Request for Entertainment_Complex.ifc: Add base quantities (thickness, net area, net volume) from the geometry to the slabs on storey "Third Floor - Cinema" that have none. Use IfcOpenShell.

First a look at what the model holds.

```python
import ifcopenshell
import ifcopenshell.util.element
import ifcopenshell.util.unit

model = ifcopenshell.open("Entertainment_Complex.ifc")
print(model.schema)
for unit_type in ("LENGTHUNIT", "AREAUNIT", "VOLUMEUNIT"):
    print(unit_type, ifcopenshell.util.unit.calculate_unit_scale(model, unit_type))
storey = next(s for s in model.by_type("IfcBuildingStorey") if s.Name == "Third Floor - Cinema")
slabs = [e for e in ifcopenshell.util.element.get_decomposition(storey) if e.is_a("IfcSlab")]
for e in sorted(slabs, key=lambda e: e.id()):
    print(e.id(), e.is_a(), e.Name, list(ifcopenshell.util.element.get_psets(e, qtos_only=True)), sep=" | ")
```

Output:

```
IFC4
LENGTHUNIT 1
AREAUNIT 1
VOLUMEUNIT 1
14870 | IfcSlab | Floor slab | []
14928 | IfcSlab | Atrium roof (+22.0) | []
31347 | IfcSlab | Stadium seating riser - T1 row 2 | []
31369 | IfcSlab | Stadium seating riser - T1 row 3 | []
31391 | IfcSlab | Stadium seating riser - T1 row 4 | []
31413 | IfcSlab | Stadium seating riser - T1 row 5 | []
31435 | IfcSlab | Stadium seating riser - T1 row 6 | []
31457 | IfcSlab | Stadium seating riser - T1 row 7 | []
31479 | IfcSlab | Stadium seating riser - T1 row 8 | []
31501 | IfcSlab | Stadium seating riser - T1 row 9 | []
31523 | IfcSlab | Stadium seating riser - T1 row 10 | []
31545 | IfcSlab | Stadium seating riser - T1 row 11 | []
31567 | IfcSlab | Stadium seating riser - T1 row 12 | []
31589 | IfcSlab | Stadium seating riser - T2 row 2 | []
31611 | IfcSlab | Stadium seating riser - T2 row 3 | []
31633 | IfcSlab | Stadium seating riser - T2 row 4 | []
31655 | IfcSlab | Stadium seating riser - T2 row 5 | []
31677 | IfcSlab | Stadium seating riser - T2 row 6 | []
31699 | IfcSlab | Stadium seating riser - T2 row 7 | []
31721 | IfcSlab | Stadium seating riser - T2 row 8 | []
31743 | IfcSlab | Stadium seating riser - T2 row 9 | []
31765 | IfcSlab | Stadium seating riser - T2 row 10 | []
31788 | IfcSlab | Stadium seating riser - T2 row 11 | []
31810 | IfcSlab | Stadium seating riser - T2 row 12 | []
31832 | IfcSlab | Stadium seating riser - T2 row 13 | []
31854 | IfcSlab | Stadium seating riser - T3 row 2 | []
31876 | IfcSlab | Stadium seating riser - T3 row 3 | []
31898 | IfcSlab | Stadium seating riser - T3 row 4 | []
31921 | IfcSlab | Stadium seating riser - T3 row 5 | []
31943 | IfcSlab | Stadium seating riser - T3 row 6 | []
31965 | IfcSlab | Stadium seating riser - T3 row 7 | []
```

```python
import ifcopenshell
import ifcopenshell.api.pset
import ifcopenshell.geom
import ifcopenshell.util.element
import ifcopenshell.util.shape
import ifcopenshell.util.unit

model = ifcopenshell.open("Entertainment_Complex.ifc")
unit_scale = ifcopenshell.util.unit.calculate_unit_scale(model)
area_scale = ifcopenshell.util.unit.calculate_unit_scale(model, "AREAUNIT")
volume_scale = ifcopenshell.util.unit.calculate_unit_scale(model, "VOLUMEUNIT")
settings = ifcopenshell.geom.settings()

storey = next(s for s in model.by_type("IfcBuildingStorey") if s.Name == "Third Floor - Cinema")
slabs = [e for e in ifcopenshell.util.element.get_decomposition(storey) if e.is_a("IfcSlab")]

for e in sorted(slabs, key=lambda e: e.id()):
    if ifcopenshell.util.element.get_psets(e, qtos_only=True, should_inherit=False):
        continue
    # Geometry comes back in metres, in the element's own axes.
    shape = ifcopenshell.geom.create_shape(settings, e)
    values = {
        "Width": ifcopenshell.util.shape.get_z(shape.geometry) / unit_scale,
        "NetArea": ifcopenshell.util.shape.get_footprint_area(shape.geometry) / area_scale,
        "NetVolume": ifcopenshell.util.shape.get_volume(shape.geometry) / volume_scale,
    }
    qto = ifcopenshell.api.pset.add_qto(model, product=e, name="Qto_SlabBaseQuantities")
    ifcopenshell.api.pset.edit_qto(model, qto=qto, properties=values)
    print(e.id(), {k: round(v, 3) for k, v in values.items()})

model.write("Entertainment_Complex-out.ifc")
```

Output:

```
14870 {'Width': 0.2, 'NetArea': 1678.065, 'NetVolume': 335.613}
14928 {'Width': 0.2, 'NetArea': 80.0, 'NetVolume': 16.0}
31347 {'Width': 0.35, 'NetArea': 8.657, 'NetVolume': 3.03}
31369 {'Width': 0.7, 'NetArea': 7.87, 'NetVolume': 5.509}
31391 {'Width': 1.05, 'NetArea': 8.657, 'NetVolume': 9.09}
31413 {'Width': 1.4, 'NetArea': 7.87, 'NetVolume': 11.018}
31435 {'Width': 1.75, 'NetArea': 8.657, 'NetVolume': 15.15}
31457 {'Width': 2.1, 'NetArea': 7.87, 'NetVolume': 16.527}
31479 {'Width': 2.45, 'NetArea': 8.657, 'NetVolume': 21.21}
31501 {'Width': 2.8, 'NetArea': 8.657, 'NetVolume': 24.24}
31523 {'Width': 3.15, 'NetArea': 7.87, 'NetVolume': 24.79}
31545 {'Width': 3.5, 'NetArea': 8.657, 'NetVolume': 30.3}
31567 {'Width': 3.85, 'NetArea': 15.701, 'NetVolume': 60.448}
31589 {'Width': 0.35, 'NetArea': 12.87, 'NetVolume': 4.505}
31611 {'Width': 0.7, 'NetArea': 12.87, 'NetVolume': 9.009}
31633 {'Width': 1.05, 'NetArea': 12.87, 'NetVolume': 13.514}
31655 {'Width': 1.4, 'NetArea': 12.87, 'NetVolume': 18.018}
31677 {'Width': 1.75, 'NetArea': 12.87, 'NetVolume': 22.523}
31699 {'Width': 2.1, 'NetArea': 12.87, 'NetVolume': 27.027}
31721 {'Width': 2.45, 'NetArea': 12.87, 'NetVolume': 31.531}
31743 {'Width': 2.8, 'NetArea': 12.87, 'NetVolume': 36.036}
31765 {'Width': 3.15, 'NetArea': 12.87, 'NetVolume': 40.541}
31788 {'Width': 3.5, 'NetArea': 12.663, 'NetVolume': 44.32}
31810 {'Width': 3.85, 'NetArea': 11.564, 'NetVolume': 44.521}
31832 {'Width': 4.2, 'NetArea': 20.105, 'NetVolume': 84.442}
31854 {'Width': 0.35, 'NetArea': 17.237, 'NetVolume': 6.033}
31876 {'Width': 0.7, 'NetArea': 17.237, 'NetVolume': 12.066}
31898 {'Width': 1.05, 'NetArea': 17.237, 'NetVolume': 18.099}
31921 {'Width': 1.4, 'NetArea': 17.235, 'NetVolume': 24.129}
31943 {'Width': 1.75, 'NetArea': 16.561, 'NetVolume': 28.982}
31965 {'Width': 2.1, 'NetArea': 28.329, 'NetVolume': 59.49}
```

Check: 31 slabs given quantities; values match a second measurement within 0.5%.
